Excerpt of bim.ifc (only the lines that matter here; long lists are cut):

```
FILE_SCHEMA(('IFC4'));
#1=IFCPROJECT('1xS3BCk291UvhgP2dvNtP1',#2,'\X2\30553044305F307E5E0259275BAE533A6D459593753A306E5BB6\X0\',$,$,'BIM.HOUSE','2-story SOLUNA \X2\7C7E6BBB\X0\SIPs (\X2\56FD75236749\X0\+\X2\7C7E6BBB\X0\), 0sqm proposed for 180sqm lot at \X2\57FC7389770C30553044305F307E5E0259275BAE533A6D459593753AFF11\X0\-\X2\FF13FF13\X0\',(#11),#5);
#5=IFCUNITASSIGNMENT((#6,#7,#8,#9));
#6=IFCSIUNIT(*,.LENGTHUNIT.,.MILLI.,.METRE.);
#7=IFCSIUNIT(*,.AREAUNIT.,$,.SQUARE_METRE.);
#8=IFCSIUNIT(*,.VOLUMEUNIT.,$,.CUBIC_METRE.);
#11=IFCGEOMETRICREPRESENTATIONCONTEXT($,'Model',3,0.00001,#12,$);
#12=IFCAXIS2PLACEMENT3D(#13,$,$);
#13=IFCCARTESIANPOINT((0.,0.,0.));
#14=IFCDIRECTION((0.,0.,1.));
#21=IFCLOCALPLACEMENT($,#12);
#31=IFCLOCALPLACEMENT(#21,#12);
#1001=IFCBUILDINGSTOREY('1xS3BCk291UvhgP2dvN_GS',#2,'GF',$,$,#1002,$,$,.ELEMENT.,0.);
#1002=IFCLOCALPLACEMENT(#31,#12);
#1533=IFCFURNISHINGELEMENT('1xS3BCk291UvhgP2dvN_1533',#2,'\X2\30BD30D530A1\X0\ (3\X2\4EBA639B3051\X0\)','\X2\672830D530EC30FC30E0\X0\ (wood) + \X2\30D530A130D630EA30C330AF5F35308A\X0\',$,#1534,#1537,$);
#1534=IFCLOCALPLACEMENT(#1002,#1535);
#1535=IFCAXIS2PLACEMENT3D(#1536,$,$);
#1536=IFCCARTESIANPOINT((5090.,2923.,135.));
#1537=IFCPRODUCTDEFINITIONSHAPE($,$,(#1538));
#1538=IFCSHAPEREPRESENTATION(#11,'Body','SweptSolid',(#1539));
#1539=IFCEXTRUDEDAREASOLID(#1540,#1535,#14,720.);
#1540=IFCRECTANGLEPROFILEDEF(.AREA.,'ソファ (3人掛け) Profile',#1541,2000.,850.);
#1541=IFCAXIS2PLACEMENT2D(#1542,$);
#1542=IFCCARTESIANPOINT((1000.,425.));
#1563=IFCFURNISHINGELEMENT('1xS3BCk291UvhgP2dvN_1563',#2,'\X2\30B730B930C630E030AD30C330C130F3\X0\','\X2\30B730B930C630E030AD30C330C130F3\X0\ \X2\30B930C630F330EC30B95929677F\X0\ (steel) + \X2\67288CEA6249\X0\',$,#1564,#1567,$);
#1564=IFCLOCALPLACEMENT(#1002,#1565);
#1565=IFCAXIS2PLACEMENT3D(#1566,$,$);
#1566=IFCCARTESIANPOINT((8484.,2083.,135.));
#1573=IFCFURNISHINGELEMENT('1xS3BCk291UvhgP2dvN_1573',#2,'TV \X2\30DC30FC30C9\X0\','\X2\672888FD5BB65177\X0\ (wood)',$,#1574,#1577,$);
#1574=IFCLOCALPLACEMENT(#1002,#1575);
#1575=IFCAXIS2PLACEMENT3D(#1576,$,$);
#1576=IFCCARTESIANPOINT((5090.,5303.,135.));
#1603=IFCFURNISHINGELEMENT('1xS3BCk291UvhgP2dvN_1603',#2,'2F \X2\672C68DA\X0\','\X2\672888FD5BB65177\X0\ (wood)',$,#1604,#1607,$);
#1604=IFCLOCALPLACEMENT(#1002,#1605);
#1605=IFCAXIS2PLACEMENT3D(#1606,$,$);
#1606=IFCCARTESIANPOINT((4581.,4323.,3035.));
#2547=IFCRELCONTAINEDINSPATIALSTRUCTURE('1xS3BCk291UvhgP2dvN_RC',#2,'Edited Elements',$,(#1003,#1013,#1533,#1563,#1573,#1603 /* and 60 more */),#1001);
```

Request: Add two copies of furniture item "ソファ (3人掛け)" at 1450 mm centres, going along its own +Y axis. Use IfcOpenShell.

```python
import ifcopenshell
import ifcopenshell.api.geometry
import ifcopenshell.api.root
import ifcopenshell.util.element
import ifcopenshell.util.placement

model = ifcopenshell.open("bim.ifc")


def reuse_history(source, copy):
    """copy_class also copies each property set's owner history, people and application; keep the originals."""
    for rel in copy.IsDefinedBy:
        if rel.is_a("IfcRelDefinesByProperties") and (history := rel.RelatingPropertyDefinition.OwnerHistory):
            rel.RelatingPropertyDefinition.OwnerHistory = source.OwnerHistory
            ifcopenshell.util.element.remove_deep2(model, history)


source = model.by_id(1533)
base = ifcopenshell.util.placement.get_local_placement(source.ObjectPlacement)
step = base[:3, 1] * 1450.0

for i in range(1, 3):
    copy = ifcopenshell.api.root.copy_class(model, product=source)
    copy.Representation = ifcopenshell.util.element.copy_deep(
        model, source.Representation, exclude=["IfcGeometricRepresentationContext", "IfcRepresentationMap"]
    )
    reuse_history(source, copy)
    matrix = base.copy()
    matrix[:3, 3] += i * step
    print("added at", matrix[:3, 3].round(3) + 0.0)
    ifcopenshell.api.geometry.edit_object_placement(model, product=copy, matrix=matrix, is_si=False)

model.write("bim_updated.ifc")
```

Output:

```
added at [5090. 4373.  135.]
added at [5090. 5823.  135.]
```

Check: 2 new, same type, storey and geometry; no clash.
